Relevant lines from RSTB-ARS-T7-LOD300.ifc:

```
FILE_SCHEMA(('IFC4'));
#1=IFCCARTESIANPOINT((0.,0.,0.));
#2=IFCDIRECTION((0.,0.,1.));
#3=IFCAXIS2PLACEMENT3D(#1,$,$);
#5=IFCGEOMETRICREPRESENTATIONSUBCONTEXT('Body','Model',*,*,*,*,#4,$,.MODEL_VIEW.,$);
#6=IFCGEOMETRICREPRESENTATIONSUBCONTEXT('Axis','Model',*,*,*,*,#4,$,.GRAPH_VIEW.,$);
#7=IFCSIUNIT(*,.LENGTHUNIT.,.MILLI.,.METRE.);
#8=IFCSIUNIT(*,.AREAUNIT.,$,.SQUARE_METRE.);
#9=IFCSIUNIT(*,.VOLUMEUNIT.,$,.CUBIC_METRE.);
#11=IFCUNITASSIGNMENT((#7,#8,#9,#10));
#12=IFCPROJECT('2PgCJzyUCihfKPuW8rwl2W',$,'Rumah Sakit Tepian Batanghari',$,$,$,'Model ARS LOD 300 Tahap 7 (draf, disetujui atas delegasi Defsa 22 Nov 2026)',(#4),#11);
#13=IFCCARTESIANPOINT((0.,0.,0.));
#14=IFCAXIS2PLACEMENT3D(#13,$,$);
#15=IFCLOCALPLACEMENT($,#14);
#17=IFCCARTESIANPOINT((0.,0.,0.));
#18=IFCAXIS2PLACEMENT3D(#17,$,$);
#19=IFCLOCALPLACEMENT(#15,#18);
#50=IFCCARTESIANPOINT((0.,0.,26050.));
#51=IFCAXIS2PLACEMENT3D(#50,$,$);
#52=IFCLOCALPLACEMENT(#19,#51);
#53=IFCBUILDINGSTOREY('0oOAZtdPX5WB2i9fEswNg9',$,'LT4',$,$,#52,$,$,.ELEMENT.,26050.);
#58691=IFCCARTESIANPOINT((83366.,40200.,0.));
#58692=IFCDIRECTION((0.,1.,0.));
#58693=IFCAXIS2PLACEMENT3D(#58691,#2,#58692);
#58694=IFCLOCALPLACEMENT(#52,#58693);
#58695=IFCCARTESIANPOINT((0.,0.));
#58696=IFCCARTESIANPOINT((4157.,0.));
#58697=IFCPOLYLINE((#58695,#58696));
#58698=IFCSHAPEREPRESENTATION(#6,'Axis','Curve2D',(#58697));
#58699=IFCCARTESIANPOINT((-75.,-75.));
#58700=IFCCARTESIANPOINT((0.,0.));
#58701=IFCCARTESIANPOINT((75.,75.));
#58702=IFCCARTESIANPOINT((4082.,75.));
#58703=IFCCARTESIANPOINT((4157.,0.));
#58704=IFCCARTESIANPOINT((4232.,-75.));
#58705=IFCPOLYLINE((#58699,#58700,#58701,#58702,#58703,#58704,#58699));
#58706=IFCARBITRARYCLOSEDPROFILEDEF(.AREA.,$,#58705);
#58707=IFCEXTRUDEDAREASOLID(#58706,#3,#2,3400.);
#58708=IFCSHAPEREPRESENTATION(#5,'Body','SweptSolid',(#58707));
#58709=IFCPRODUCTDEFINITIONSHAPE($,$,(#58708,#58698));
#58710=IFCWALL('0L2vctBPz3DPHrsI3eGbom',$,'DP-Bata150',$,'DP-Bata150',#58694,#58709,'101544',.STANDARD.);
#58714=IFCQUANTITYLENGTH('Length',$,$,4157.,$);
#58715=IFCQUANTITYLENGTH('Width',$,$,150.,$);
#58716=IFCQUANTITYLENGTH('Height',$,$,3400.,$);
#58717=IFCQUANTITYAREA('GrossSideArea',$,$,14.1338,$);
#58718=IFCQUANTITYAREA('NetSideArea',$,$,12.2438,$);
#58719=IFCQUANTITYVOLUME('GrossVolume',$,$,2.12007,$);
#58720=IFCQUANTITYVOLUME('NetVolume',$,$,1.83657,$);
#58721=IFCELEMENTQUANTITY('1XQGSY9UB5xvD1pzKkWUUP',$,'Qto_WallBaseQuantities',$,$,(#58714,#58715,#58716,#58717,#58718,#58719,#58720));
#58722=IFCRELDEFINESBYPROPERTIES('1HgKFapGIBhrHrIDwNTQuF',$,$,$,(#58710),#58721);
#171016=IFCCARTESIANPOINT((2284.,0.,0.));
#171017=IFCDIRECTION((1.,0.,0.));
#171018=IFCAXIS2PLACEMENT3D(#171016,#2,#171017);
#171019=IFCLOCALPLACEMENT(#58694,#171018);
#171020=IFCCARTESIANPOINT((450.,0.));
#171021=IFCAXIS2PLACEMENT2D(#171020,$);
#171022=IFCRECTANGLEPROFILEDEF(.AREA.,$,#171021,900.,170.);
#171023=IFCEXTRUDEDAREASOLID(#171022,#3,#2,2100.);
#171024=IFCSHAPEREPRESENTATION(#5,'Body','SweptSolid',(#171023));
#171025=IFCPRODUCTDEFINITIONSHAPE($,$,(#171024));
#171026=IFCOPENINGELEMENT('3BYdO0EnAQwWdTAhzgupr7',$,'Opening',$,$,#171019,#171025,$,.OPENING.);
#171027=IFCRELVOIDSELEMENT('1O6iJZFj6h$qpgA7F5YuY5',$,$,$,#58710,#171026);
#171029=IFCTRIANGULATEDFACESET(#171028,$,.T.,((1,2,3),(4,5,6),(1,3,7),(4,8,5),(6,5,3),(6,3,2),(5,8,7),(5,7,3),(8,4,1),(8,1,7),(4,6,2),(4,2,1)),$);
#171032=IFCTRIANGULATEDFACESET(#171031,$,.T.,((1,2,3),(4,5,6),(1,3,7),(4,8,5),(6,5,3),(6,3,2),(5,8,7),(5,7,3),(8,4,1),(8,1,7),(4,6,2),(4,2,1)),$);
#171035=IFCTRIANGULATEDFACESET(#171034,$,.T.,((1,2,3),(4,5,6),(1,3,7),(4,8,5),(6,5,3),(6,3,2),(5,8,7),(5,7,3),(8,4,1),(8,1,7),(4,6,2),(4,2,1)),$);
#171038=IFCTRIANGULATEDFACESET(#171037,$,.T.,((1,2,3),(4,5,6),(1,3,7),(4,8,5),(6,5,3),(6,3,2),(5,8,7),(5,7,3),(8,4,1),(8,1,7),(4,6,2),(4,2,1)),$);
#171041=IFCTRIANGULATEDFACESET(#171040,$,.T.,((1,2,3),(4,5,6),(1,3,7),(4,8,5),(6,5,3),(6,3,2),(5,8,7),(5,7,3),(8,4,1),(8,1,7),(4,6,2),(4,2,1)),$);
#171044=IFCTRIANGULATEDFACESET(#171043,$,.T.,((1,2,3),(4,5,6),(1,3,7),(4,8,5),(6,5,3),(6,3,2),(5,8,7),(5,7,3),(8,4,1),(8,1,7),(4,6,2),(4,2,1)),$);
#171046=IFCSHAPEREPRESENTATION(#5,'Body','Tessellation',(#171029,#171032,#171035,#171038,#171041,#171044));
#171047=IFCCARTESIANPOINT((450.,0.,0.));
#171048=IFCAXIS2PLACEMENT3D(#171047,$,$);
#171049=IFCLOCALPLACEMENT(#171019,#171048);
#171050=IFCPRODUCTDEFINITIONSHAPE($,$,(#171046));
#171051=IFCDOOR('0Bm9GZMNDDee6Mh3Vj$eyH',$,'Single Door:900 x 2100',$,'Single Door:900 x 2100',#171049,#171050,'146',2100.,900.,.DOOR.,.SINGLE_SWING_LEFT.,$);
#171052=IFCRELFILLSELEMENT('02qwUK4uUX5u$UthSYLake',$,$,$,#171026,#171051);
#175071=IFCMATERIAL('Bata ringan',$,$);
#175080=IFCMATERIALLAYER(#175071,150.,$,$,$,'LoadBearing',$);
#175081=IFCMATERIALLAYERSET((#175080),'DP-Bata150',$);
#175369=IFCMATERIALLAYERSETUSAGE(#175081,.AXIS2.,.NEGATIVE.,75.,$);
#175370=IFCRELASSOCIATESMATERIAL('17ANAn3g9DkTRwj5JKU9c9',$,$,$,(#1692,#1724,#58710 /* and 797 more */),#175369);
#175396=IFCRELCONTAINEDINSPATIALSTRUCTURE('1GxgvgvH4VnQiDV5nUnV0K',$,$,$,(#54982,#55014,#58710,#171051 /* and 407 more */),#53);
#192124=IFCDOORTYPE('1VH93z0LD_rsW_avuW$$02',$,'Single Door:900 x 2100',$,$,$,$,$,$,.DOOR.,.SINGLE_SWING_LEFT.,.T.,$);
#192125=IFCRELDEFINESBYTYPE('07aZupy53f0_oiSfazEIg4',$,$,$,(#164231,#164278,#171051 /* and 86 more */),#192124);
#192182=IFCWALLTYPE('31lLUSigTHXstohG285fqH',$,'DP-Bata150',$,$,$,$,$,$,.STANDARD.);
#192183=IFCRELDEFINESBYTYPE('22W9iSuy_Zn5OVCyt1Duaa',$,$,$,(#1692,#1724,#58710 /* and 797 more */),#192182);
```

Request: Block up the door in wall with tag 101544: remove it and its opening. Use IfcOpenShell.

```python
import ifcopenshell
import ifcopenshell.api.feature
import ifcopenshell.api.pset
import ifcopenshell.api.root
import ifcopenshell.geom
import ifcopenshell.util.element
import ifcopenshell.util.shape
import ifcopenshell.util.unit

model = ifcopenshell.open("RSTB-ARS-T7-LOD300.ifc")
area_scale = ifcopenshell.util.unit.calculate_unit_scale(model, "AREAUNIT")
volume_scale = ifcopenshell.util.unit.calculate_unit_scale(model, "VOLUMEUNIT")
settings = ifcopenshell.geom.settings()


def volume(element):
    """Net volume in cubic metres, openings subtracted."""
    shape = ifcopenshell.geom.create_shape(settings, element)
    return ifcopenshell.util.shape.get_volume(shape.geometry)


door = model.by_guid("0Bm9GZMNDDee6Mh3Vj$eyH")
opening = door.FillsVoids[0].RelatingOpeningElement
wall = opening.VoidsElements[0].RelatingBuildingElement
before = volume(wall)

ifcopenshell.api.root.remove_product(model, product=door)
ifcopenshell.api.feature.remove_feature(model, feature=opening)

after = volume(wall)
thickness = 0.15  # wall thickness in metres

# Update the wall's stored quantities.
qto = model.by_id(ifcopenshell.util.element.get_pset(wall, "Qto_WallBaseQuantities", should_inherit=False)["id"])
ifcopenshell.api.pset.edit_qto(model, qto=qto, properties={
    "NetSideArea": after / thickness / area_scale,
    "NetVolume": after / volume_scale,
})

print(f"wall volume {before:.3f} -> {after:.3f} m3")

model.write("RSTB-ARS-T7-LOD300_edited.ifc")
```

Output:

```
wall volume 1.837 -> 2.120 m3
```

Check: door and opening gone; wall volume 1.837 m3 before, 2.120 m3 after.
